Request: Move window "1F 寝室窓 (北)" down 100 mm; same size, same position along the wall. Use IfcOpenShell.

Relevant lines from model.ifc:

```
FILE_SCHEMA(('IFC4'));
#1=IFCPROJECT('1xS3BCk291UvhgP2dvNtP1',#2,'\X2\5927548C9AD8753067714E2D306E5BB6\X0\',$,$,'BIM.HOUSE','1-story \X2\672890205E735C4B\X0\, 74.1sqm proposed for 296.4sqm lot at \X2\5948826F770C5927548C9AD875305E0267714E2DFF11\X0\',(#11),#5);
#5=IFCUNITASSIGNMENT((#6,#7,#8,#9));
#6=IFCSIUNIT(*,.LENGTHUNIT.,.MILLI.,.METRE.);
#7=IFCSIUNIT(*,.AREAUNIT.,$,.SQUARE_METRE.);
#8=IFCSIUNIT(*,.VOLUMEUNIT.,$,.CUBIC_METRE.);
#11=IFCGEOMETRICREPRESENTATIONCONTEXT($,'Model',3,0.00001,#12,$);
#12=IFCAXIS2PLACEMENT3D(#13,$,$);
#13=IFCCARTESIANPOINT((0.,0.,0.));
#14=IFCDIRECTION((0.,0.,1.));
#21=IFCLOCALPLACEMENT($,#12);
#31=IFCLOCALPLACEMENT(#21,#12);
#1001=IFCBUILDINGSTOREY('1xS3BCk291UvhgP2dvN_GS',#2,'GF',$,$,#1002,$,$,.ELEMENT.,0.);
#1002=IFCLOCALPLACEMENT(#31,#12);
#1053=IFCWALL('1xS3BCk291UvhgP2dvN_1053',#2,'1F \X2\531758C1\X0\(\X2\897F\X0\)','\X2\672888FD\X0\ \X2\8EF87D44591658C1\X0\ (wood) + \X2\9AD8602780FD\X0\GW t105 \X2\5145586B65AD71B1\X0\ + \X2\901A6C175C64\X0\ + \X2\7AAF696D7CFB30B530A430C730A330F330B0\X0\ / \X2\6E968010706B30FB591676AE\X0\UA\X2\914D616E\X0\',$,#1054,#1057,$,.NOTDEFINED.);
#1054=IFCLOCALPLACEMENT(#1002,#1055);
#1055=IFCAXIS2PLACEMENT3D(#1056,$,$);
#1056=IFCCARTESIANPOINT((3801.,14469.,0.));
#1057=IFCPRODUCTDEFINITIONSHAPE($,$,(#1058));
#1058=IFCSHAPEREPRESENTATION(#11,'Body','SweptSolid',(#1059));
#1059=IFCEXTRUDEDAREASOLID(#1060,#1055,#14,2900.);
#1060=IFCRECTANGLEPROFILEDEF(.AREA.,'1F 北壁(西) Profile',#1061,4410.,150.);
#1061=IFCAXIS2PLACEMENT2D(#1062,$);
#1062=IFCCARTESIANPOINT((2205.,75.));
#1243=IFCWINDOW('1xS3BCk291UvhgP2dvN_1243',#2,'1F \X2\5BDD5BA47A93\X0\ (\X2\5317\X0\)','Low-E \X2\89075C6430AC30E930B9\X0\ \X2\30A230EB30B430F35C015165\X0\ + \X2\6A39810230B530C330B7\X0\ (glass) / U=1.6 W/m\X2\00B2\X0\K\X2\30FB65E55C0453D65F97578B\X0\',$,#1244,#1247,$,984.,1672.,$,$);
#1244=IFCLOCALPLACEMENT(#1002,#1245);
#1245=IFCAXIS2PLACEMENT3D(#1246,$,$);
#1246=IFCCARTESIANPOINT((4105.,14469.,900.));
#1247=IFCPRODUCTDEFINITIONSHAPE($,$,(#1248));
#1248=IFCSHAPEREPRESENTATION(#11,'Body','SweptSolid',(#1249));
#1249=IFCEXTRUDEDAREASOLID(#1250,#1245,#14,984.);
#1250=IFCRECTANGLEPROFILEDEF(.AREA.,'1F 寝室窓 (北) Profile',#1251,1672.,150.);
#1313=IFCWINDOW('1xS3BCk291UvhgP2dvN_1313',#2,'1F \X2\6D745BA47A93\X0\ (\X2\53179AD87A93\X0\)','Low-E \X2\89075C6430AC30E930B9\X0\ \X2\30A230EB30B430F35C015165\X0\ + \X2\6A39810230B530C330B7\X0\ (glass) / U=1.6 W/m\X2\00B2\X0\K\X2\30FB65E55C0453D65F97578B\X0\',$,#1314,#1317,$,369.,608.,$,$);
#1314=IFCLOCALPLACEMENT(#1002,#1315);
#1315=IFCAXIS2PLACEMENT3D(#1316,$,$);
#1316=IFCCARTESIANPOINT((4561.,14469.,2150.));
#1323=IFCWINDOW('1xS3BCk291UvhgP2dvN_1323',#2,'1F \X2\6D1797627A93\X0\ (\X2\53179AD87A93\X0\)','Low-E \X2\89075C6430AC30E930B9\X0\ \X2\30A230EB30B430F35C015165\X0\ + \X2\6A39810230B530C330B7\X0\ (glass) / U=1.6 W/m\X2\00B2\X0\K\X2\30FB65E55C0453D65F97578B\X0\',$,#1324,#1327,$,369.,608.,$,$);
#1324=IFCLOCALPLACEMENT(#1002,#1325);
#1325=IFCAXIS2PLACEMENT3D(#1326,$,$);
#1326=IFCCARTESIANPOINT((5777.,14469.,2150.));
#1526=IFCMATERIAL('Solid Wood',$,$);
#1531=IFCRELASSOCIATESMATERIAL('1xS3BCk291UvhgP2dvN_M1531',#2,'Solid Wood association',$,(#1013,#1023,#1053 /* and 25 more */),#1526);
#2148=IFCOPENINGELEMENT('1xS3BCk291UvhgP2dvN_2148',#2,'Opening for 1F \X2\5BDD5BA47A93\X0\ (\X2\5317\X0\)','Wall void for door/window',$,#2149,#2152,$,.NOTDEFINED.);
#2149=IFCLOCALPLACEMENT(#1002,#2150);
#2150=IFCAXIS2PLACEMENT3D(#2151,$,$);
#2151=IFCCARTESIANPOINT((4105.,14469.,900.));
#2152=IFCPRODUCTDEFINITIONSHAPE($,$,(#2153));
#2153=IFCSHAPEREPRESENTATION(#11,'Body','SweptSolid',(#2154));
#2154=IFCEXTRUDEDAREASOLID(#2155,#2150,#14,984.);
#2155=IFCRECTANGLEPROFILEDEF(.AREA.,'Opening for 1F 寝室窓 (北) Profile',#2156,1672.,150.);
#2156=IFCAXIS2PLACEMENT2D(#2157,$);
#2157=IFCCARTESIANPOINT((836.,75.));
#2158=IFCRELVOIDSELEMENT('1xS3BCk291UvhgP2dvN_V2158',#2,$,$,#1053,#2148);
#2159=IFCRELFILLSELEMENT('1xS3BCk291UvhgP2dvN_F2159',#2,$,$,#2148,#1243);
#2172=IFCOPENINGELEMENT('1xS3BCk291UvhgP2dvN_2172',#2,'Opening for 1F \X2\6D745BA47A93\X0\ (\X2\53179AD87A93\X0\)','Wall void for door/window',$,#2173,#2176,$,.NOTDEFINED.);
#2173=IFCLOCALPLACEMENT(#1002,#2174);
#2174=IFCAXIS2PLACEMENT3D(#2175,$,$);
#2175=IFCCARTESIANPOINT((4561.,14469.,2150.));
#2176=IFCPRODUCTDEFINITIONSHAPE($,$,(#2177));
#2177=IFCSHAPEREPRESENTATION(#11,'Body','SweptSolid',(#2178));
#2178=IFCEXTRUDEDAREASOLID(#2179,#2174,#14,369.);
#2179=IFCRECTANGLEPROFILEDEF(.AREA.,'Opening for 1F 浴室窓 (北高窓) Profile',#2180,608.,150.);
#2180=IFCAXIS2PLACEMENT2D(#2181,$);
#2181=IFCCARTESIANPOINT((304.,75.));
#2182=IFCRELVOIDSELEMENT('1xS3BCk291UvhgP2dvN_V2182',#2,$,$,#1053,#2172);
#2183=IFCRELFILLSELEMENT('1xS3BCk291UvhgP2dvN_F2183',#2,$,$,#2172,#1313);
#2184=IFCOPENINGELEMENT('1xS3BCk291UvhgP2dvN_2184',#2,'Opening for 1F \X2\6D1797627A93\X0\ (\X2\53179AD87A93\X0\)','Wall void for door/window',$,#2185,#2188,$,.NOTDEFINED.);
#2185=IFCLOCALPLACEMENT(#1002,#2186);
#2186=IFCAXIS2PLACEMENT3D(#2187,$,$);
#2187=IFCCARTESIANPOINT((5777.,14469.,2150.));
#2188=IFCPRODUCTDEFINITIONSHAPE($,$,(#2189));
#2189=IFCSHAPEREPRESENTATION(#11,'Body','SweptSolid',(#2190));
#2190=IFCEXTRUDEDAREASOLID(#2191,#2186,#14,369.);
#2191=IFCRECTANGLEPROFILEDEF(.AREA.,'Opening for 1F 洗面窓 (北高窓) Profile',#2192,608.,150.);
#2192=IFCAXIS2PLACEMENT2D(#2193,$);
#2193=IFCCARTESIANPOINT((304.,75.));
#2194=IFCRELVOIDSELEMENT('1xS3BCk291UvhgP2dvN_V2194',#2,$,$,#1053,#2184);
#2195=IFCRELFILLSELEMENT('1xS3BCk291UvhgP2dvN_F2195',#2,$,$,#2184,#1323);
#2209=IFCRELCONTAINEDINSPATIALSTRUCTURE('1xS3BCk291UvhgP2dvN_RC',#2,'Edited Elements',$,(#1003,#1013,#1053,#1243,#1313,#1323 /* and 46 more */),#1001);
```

```python
import numpy as np
import ifcopenshell
import ifcopenshell.api.geometry
import ifcopenshell.util.placement
import ifcopenshell.util.unit

model = ifcopenshell.open("model.ifc")
unit_scale = ifcopenshell.util.unit.calculate_unit_scale(model)

window = model.by_guid("1xS3BCk291UvhgP2dvN_1243")
opening = window.FillsVoids[0].RelatingOpeningElement
dz = -100.0

shift = np.array([0.0, 0.0, dz])
# The window is not placed relative to its opening, so move both.
for product in (opening, window):
    matrix = ifcopenshell.util.placement.get_local_placement(product.ObjectPlacement)
    matrix[:3, 3] += shift
    ifcopenshell.api.geometry.edit_object_placement(model, product=product, matrix=matrix, is_si=False)

print(f"moved by {dz * unit_scale:+.3f} m")

model.write("model_edited.ifc")
```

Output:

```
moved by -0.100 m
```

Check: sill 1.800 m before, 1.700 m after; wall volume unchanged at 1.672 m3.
